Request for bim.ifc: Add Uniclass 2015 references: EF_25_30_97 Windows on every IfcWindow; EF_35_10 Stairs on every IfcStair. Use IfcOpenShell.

First a look at what the model holds.

```python
import ifcopenshell

model = ifcopenshell.open("bim.ifc")
print(model.schema)
print("classifications:", [c.Name for c in model.by_type("IfcClassification")])
for ifc_class in ("IfcDoor", "IfcRoof", "IfcStair", "IfcWall", "IfcWindow"):
    print(ifc_class, len(model.by_type(ifc_class)))
```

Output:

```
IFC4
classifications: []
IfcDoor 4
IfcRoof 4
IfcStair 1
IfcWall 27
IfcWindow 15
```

```python
import ifcopenshell
import ifcopenshell.api.classification

model = ifcopenshell.open("bim.ifc")

system = ifcopenshell.api.classification.add_classification(model, classification="Uniclass 2015")

codes = {
    "IfcWindow": ("EF_25_30_97", "Windows"),
    "IfcStair": ("EF_35_10", "Stairs"),
}
for ifc_class, (code, name) in codes.items():
    products = model.by_type(ifc_class)
    ifcopenshell.api.classification.add_reference(
        model, products=products, classification=system, identification=code, name=name
    )
    print(code, len(products))

model.write("bim_v2.ifc")
```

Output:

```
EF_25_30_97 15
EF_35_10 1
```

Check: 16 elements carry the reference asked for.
